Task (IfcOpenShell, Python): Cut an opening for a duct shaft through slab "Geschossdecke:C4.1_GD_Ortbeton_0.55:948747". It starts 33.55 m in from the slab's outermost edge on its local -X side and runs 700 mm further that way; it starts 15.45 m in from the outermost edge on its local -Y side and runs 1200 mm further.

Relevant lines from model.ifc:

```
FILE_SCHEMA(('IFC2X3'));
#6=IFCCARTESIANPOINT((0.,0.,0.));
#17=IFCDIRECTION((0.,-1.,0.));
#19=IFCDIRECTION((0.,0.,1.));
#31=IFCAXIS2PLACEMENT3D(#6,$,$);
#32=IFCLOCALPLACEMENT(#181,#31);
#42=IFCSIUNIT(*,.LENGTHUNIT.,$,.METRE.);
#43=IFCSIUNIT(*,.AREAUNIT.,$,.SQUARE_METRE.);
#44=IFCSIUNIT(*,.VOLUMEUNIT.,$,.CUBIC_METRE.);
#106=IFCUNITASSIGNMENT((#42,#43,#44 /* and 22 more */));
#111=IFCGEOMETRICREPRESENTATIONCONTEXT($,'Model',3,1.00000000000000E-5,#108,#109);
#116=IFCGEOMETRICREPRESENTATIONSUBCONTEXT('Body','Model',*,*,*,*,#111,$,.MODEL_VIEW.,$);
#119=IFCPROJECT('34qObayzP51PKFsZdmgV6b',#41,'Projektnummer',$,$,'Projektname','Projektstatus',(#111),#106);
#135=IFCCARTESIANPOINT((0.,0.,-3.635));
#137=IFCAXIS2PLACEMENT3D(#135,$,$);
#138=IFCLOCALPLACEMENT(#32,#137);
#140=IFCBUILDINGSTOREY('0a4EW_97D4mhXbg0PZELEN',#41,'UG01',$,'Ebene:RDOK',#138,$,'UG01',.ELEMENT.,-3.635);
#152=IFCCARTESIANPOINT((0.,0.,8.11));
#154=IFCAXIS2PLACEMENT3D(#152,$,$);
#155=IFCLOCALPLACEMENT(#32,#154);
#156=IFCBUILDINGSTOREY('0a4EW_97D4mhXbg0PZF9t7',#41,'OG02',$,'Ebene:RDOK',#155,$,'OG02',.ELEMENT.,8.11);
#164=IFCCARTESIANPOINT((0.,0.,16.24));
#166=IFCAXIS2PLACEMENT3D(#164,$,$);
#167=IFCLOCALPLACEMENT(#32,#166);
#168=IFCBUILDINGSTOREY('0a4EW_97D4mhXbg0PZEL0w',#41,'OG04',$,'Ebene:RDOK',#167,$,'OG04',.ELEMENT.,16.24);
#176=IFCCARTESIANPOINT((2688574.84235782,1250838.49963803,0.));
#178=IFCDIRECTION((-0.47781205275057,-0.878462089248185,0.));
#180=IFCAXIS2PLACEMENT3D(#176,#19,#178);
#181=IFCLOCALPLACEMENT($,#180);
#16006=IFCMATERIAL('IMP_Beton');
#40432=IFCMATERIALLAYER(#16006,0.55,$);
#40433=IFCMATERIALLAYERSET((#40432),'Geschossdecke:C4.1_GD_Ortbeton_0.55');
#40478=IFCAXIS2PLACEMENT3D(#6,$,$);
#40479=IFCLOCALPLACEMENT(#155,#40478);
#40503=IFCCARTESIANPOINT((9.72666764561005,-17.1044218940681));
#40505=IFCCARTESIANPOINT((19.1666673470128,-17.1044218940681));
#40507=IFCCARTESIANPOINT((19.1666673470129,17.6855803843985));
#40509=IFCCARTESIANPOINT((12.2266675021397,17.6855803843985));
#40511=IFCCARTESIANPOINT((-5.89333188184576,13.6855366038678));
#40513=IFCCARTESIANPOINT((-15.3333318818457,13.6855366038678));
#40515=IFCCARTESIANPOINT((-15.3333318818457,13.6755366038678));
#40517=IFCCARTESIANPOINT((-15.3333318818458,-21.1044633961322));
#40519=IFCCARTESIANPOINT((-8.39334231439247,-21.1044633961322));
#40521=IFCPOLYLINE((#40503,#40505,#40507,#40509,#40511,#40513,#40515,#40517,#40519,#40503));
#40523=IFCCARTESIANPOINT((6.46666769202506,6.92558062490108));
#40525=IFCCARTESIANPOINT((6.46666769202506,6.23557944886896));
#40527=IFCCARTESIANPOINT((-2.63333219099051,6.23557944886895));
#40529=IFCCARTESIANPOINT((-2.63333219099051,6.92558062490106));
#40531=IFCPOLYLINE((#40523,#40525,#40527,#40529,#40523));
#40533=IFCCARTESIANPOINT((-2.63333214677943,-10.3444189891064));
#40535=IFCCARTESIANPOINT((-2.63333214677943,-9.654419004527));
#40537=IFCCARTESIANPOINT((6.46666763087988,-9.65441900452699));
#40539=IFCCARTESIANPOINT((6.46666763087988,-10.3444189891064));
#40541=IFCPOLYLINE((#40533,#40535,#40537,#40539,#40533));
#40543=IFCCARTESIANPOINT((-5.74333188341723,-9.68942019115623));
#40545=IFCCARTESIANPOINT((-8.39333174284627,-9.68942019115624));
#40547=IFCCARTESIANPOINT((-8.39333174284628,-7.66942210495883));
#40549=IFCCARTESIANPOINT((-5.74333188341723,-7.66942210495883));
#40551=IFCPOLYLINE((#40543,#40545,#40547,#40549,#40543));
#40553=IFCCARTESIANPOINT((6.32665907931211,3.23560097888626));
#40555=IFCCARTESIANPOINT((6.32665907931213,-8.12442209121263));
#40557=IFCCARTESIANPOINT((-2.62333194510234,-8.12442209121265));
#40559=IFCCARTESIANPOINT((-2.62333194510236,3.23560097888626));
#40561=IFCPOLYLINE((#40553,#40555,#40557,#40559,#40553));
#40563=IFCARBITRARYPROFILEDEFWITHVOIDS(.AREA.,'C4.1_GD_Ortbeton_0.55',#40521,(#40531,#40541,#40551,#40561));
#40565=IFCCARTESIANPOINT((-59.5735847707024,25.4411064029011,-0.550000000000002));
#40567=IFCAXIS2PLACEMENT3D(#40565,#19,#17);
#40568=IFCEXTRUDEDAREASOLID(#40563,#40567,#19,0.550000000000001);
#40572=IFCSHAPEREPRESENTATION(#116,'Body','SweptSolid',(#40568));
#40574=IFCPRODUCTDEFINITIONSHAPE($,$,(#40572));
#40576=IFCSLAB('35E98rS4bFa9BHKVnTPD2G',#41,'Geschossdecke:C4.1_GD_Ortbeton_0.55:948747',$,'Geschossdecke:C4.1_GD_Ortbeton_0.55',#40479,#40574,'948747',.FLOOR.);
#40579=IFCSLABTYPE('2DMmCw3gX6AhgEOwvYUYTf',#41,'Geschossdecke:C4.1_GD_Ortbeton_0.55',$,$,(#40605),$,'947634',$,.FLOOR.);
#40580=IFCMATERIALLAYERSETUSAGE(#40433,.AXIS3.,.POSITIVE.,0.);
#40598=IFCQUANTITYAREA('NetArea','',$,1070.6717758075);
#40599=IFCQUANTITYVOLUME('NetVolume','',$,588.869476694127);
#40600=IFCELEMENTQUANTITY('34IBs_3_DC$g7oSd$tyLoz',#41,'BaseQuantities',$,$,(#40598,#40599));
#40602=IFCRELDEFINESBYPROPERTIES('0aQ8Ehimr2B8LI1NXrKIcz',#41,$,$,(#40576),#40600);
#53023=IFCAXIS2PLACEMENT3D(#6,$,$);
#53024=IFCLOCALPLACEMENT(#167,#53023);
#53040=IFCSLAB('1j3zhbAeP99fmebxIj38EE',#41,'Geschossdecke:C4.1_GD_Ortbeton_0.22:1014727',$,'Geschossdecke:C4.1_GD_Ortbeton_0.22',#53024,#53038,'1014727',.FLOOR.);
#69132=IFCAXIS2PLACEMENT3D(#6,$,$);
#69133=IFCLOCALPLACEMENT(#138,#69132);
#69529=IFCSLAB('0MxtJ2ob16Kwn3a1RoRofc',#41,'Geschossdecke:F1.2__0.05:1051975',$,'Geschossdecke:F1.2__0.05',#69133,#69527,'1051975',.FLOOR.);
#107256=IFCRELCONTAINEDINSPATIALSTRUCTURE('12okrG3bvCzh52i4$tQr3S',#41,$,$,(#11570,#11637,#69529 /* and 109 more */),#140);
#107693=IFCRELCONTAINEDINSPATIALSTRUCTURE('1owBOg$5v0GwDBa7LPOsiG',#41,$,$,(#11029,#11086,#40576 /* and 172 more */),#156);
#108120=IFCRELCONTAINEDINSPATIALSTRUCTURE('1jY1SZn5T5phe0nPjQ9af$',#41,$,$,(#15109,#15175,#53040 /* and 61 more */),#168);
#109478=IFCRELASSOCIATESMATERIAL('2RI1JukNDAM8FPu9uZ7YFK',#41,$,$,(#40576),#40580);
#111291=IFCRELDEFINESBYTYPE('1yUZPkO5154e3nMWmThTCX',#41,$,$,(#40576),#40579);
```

```python
import numpy as np
import ifcopenshell
import ifcopenshell.api.feature
import ifcopenshell.api.geometry
import ifcopenshell.api.pset
import ifcopenshell.api.root
import ifcopenshell.geom
import ifcopenshell.util.element
import ifcopenshell.util.placement
import ifcopenshell.util.representation
import ifcopenshell.util.shape
import ifcopenshell.util.unit

model = ifcopenshell.open("model.ifc")
unit_scale = ifcopenshell.util.unit.calculate_unit_scale(model)
area_scale = ifcopenshell.util.unit.calculate_unit_scale(model, "AREAUNIT")
volume_scale = ifcopenshell.util.unit.calculate_unit_scale(model, "VOLUMEUNIT")
settings = ifcopenshell.geom.settings()


def volume(element):
    """Net volume in cubic metres, openings subtracted."""
    shape = ifcopenshell.geom.create_shape(settings, element)
    return ifcopenshell.util.shape.get_volume(shape.geometry)


slab = model.by_guid("35E98rS4bFa9BHKVnTPD2G")
before = volume(slab)

# Extent in the slab's own axes, in metres. The edges named are its -X and -Y sides.
slab_shape = ifcopenshell.geom.create_shape(settings, slab)
vertices = ifcopenshell.util.shape.get_vertices(slab_shape.geometry)
x_min, y_min, bottom = vertices.min(axis=0)
top = vertices[:, 2].max()

opening = ifcopenshell.api.root.create_entity(model, ifc_class="IfcOpeningElement", name="Duct shaft opening")
context = ifcopenshell.util.representation.get_context(model, "Model", "Body", "MODEL_VIEW")
width, depth = 0.7, 1.2
outline = [(0.0, 0.0), (width, 0.0), (width, depth), (0.0, depth), (0.0, 0.0)]
# Overshoot both faces by 50 mm so the cut is clean.
shape = ifcopenshell.api.geometry.add_slab_representation(
    model, context=context, depth=top - bottom + 0.1, polyline=outline
)
ifcopenshell.api.geometry.assign_representation(model, product=opening, representation=shape)

matrix = ifcopenshell.util.placement.get_local_placement(slab.ObjectPlacement)
matrix[:, 3] = matrix @ np.append(np.array([x_min + 33.55, y_min + 15.45, bottom - 0.05]) / unit_scale, 1.0)
ifcopenshell.api.geometry.edit_object_placement(model, product=opening, matrix=matrix, is_si=False)
ifcopenshell.api.feature.add_feature(model, feature=opening, element=slab)

after = volume(slab)

# Update the slab's stored quantities.
qto = model.by_id(ifcopenshell.util.element.get_pset(slab, "BaseQuantities", should_inherit=False)["id"])
ifcopenshell.api.pset.edit_qto(model, qto=qto, properties={
    "NetArea": after / (top - bottom) / area_scale,
    "NetVolume": after / volume_scale,
})

print(f"slab volume {before:.3f} -> {after:.3f} m3")

model.write("model_v2.ifc")
```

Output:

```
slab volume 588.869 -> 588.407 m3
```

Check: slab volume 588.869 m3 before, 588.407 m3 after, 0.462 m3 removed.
